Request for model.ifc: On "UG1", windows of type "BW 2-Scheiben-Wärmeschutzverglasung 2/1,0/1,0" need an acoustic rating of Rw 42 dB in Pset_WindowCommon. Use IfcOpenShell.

First a look at what the model holds.

```python
import ifcopenshell
import ifcopenshell.util.element

model = ifcopenshell.open("model.ifc")
print(model.schema)
storey = next(s for s in model.by_type("IfcBuildingStorey") if s.Name == "UG1")
windows = [e for e in ifcopenshell.util.element.get_decomposition(storey) if e.is_a("IfcWindow")]
seen = {}
for e in windows:
    element_type = ifcopenshell.util.element.get_type(e)
    key = (element_type.Name if element_type != e and element_type else None, ifcopenshell.util.element.get_pset(e, "Pset_WindowCommon", "AcousticRating"))
    seen[key] = seen.get(key, 0) + 1
for (name, value), count in sorted(seen.items(), key=str):
    print(count, "x", name, "|", value)
```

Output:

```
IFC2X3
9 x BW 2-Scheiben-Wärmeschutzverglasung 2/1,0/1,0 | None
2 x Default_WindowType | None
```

```python
import ifcopenshell
import ifcopenshell.api.pset
import ifcopenshell.util.element

model = ifcopenshell.open("model.ifc")

storey = next(s for s in model.by_type("IfcBuildingStorey") if s.Name == "UG1")
windows = [e for e in ifcopenshell.util.element.get_decomposition(storey) if e.is_a("IfcWindow")]

count = 0
for e in windows:
    element_type = ifcopenshell.util.element.get_type(e)
    if element_type in (None, e) or element_type.Name != "BW 2-Scheiben-Wärmeschutzverglasung 2/1,0/1,0":
        continue
    # add_pset returns the element's existing set when there is one.
    pset = ifcopenshell.api.pset.add_pset(model, product=e, name="Pset_WindowCommon")
    ifcopenshell.api.pset.edit_pset(model, pset=pset, properties={"AcousticRating": "Rw 42 dB"})
    count += 1

print(count, "windows updated")

model.write("model_rev.ifc")
```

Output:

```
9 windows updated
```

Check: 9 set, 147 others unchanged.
